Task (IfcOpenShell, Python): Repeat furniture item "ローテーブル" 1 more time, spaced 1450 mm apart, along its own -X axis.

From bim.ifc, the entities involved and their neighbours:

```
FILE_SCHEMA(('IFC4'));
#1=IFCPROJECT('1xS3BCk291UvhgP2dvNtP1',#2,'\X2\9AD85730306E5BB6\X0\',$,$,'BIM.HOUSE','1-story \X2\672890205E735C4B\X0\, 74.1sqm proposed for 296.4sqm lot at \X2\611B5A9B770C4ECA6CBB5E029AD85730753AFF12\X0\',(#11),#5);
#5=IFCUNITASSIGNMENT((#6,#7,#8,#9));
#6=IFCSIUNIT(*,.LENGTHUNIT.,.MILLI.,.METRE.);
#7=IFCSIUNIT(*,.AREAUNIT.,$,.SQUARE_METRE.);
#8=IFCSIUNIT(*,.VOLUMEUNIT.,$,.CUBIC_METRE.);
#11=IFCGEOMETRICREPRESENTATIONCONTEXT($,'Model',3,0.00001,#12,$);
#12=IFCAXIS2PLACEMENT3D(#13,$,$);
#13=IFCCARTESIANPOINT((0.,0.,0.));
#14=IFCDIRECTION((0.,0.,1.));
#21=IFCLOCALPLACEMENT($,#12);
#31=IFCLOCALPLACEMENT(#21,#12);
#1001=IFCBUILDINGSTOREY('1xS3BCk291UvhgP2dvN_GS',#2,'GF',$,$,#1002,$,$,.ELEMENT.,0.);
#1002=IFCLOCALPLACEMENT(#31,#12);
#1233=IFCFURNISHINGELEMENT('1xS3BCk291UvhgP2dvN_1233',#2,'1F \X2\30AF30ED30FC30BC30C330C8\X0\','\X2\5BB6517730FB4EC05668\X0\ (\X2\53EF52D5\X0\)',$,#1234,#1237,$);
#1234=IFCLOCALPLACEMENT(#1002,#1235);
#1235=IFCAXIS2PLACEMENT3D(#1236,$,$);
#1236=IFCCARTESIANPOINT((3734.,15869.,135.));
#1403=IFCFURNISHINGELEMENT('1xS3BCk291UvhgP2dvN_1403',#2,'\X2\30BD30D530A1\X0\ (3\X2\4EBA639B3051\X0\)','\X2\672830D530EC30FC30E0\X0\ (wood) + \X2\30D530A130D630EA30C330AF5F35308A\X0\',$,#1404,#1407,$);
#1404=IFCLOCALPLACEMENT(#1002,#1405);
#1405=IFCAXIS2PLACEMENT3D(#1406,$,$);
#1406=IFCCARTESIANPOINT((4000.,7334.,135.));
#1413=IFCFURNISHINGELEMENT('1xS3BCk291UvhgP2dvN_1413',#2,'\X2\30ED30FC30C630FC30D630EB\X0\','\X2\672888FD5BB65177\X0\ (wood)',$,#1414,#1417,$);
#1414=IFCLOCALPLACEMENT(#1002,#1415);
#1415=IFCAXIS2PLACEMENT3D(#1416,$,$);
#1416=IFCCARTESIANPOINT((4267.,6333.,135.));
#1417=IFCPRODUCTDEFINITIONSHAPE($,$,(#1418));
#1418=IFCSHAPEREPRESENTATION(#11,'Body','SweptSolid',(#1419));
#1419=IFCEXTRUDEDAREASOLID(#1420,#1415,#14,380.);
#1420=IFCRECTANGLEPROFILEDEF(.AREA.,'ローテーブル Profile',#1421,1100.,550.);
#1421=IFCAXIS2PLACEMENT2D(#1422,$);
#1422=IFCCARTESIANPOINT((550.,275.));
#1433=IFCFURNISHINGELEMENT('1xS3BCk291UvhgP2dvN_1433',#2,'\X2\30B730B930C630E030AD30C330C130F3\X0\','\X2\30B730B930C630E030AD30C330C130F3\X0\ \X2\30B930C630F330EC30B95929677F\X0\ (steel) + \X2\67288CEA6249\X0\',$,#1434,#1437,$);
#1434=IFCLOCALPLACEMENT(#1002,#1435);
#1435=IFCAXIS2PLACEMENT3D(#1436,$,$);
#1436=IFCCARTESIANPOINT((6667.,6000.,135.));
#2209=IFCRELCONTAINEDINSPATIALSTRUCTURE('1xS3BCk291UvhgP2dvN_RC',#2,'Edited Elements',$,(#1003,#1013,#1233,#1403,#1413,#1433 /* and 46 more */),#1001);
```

```python
import ifcopenshell
import ifcopenshell.api.geometry
import ifcopenshell.api.root
import ifcopenshell.util.element
import ifcopenshell.util.placement
import ifcopenshell.util.unit

model = ifcopenshell.open("bim.ifc")
unit_scale = ifcopenshell.util.unit.calculate_unit_scale(model)


def reuse_history(source, copy):
    """copy_class also copies each property set's owner history, people and application; keep the originals."""
    for rel in copy.IsDefinedBy:
        if rel.is_a("IfcRelDefinesByProperties") and (history := rel.RelatingPropertyDefinition.OwnerHistory):
            rel.RelatingPropertyDefinition.OwnerHistory = source.OwnerHistory
            ifcopenshell.util.element.remove_deep2(model, history)


source = model.by_id(1413)
base = ifcopenshell.util.placement.get_local_placement(source.ObjectPlacement)
step = -base[:3, 0] * 1.45 / unit_scale

for i in range(1, 2):
    copy = ifcopenshell.api.root.copy_class(model, product=source)
    copy.Representation = ifcopenshell.util.element.copy_deep(
        model, source.Representation, exclude=["IfcGeometricRepresentationContext", "IfcRepresentationMap"]
    )
    reuse_history(source, copy)
    matrix = base.copy()
    matrix[:3, 3] += i * step
    print("added at", matrix[:3, 3].round(3) + 0.0)
    ifcopenshell.api.geometry.edit_object_placement(model, product=copy, matrix=matrix, is_si=False)

model.write("bim_edited.ifc")
```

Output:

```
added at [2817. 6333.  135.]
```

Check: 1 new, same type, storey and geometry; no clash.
